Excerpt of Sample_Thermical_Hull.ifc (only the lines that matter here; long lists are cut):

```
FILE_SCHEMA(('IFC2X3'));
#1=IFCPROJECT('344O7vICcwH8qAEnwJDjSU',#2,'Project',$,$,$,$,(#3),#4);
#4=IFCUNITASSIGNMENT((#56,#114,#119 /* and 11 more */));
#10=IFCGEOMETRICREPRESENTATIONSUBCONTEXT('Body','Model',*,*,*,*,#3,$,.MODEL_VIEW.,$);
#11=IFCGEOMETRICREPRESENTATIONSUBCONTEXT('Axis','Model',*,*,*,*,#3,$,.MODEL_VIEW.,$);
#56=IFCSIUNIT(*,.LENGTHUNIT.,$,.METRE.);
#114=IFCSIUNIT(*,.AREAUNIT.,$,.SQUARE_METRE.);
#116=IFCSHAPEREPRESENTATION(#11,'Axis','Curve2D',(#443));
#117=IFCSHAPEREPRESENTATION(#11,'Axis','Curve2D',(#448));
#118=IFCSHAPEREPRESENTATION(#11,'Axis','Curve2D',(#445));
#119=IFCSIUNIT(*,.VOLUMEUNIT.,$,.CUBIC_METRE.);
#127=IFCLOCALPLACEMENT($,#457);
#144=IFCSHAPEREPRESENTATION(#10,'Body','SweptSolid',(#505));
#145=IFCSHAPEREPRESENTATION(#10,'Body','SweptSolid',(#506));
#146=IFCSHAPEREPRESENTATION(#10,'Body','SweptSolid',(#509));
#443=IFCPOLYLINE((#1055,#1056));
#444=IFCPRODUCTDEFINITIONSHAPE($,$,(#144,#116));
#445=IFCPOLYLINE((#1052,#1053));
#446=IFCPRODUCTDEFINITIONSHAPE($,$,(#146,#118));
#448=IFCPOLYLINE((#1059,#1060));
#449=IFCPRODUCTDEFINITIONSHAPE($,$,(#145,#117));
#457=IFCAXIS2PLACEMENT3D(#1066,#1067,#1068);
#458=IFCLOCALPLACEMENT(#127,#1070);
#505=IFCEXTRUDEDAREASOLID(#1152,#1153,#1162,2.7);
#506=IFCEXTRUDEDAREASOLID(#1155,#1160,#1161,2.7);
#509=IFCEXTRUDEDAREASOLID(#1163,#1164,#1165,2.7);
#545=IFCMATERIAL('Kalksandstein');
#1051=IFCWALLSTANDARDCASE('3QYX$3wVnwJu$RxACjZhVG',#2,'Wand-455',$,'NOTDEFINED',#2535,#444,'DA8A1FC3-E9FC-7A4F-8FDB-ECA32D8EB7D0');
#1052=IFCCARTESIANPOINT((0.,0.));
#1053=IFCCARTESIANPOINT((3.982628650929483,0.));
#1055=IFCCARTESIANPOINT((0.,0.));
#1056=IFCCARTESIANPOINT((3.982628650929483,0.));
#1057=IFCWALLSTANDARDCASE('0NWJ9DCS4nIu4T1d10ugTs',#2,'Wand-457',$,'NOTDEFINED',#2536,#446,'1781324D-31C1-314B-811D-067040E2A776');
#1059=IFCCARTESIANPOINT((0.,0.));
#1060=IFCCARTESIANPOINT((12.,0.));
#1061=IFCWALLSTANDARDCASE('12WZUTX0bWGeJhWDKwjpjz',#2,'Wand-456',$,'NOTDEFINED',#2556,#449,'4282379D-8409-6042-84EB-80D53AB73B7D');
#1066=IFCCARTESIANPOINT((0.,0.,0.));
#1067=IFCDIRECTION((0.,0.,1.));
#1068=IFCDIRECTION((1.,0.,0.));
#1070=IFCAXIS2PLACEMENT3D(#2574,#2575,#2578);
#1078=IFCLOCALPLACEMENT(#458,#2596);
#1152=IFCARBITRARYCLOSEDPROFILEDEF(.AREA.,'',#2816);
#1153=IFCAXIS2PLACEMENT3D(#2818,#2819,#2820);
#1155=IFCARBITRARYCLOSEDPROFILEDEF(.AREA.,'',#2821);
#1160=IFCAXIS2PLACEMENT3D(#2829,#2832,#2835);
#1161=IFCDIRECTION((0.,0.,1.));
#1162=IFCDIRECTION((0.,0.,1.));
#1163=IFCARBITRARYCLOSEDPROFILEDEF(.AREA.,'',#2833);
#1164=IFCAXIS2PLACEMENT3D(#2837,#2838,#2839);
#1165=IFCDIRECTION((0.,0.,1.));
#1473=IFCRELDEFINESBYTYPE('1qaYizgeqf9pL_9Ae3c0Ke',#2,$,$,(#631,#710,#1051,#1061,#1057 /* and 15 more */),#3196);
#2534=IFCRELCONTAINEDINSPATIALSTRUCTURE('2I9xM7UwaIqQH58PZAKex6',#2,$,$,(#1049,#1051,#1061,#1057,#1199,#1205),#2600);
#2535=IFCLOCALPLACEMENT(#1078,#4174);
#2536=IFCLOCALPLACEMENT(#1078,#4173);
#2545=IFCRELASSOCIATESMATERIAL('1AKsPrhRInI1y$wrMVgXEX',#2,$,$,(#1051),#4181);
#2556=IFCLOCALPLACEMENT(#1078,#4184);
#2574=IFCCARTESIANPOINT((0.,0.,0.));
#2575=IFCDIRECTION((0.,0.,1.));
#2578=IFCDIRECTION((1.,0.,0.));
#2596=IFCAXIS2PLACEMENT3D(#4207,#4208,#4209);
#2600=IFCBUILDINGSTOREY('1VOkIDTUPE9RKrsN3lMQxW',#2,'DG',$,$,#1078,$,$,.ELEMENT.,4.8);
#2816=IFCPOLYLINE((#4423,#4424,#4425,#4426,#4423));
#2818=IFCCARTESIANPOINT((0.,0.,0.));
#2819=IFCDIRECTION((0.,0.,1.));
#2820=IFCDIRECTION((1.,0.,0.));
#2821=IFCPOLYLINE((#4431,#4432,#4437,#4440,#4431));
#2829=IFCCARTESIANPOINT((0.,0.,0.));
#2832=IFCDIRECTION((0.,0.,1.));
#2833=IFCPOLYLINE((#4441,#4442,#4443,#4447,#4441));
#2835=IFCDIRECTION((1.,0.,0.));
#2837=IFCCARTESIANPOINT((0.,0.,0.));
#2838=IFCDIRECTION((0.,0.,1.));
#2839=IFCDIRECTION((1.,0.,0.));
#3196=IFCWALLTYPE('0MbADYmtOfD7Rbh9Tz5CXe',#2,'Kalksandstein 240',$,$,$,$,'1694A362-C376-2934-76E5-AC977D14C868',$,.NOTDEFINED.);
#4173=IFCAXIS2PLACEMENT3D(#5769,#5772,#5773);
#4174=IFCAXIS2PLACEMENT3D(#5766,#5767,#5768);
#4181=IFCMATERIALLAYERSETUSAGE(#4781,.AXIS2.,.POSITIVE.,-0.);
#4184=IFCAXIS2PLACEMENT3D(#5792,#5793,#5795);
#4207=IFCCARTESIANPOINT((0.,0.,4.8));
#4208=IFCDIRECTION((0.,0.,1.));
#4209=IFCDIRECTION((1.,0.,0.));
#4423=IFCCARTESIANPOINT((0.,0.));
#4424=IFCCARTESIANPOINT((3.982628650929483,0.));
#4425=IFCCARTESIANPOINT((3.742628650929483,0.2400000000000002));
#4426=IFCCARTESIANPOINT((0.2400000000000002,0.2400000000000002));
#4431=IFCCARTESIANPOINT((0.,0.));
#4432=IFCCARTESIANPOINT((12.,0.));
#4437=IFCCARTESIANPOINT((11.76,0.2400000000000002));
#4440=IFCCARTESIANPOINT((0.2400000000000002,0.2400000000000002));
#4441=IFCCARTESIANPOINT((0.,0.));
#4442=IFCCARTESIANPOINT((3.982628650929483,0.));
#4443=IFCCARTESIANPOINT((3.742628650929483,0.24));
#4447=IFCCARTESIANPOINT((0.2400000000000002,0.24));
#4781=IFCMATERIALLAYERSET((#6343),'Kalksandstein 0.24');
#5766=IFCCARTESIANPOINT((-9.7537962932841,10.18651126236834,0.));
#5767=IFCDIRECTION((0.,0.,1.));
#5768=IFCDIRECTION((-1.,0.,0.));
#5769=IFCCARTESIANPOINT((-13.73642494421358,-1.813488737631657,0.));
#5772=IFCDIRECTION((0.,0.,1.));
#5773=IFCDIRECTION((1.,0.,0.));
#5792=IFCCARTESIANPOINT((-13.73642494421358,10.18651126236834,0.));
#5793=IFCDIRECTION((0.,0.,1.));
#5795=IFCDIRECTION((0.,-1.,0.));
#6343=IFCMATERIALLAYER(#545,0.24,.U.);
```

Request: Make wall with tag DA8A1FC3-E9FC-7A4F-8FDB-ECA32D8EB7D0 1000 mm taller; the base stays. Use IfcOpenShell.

```python
import ifcopenshell
import ifcopenshell.geom
import ifcopenshell.util.representation
import ifcopenshell.util.shape
import ifcopenshell.util.unit

model = ifcopenshell.open("Sample_Thermical_Hull.ifc")
unit_scale = ifcopenshell.util.unit.calculate_unit_scale(model)
settings = ifcopenshell.geom.settings()


def volume(element):
    """Net volume in cubic metres, openings subtracted."""
    shape = ifcopenshell.geom.create_shape(settings, element)
    return ifcopenshell.util.shape.get_volume(shape.geometry)


wall = model.by_guid("3QYX$3wVnwJu$RxACjZhVG")
before = volume(wall)

body = ifcopenshell.util.representation.get_representation(wall, "Model", "Body")
solid = body.Items[0]
old_height = solid.Depth
solid.Depth += 1 / unit_scale
after = volume(wall)

print(f"height {old_height:g} -> {solid.Depth:g}, volume {before:.3f} -> {after:.3f} m3")

model.write("Sample_Thermical_Hull_edited.ifc")
```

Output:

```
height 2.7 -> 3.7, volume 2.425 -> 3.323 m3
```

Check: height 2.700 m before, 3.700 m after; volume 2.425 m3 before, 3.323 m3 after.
